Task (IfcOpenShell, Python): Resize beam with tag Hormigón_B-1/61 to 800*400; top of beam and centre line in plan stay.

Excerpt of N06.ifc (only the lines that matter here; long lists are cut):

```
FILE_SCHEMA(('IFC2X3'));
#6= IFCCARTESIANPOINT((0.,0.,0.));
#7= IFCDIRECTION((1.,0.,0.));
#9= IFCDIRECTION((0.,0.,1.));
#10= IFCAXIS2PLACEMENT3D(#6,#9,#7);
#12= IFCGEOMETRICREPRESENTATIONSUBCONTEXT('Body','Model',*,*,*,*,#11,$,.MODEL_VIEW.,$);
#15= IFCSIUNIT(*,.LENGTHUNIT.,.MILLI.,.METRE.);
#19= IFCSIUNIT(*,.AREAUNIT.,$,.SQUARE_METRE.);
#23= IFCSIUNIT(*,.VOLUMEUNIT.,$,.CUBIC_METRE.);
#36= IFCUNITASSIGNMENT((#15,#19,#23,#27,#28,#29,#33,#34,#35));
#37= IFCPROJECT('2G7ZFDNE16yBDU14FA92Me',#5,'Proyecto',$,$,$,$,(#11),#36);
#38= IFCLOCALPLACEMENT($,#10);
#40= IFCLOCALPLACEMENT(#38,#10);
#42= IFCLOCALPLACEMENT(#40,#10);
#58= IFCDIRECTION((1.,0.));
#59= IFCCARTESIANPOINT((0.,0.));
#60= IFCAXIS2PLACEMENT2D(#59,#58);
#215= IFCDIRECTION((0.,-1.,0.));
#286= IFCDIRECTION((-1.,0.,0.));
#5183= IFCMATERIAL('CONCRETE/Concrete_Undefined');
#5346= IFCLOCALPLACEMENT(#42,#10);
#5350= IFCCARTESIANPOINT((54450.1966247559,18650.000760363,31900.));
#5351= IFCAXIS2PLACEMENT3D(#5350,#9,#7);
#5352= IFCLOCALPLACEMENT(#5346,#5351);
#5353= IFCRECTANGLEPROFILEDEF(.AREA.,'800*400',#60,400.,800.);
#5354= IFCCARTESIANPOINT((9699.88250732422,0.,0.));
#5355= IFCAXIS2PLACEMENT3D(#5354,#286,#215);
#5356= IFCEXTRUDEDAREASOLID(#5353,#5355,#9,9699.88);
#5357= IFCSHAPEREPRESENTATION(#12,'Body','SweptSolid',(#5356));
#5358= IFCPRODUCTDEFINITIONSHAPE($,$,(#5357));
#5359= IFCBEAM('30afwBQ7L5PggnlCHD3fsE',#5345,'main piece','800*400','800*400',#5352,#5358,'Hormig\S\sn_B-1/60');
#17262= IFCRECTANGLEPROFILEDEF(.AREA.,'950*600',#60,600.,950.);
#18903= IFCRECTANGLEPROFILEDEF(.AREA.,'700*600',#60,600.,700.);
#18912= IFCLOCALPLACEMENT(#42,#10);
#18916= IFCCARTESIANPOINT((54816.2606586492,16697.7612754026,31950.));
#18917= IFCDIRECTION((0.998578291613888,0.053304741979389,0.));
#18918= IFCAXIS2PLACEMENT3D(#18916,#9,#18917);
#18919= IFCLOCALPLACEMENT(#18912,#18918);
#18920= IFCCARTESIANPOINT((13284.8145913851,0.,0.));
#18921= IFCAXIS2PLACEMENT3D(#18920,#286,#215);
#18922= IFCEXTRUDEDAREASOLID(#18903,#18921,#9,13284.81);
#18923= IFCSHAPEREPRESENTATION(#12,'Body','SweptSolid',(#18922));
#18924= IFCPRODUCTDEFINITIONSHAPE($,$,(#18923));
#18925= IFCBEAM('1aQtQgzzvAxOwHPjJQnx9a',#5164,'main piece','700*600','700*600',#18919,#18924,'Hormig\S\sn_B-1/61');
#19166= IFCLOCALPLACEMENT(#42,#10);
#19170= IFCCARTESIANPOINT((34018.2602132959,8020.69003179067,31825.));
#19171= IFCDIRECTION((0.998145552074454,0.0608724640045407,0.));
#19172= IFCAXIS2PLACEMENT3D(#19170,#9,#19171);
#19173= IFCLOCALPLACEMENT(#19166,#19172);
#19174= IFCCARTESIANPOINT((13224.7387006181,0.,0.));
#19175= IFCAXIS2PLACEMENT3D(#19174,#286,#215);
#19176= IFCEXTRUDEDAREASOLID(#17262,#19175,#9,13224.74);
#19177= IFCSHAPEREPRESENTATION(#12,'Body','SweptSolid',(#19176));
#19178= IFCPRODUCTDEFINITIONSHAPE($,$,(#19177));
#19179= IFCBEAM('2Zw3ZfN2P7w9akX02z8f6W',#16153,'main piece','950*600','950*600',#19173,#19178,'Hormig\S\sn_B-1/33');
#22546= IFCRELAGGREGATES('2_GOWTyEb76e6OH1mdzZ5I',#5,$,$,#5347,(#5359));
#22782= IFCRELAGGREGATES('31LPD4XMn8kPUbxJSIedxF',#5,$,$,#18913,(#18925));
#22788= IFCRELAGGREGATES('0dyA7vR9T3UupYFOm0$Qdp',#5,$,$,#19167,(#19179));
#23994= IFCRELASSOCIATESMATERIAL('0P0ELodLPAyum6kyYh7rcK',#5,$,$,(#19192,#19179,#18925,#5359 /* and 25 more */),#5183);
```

```python
import ifcopenshell
import ifcopenshell.util.element
import ifcopenshell.util.representation

model = ifcopenshell.open("N06.ifc")

member = model.by_guid("1aQtQgzzvAxOwHPjJQnx9a")
source = next(p for p in model.by_type("IfcRectangleProfileDef") if p.ProfileName == "800*400")

body = ifcopenshell.util.representation.get_representation(member, "Model", "Body")
solid = body.Items[0]
old_profile = solid.SweptArea

# Copy the section's sizes but keep this member's own profile position.
profile = ifcopenshell.util.element.copy(model, source)
# Profiles are centred, so shift by half the change in depth to hold the top.
shift = (old_profile.YDim - profile.YDim) / 2
x, y = old_profile.Position.Location.Coordinates
up = (0.0, 1.0)  # upwards, in the solid's own plane
location = model.createIfcCartesianPoint((x + up[0] * shift, y + up[1] * shift))
profile.Position = model.createIfcAxis2Placement2D(location, old_profile.Position.RefDirection)
solid.SweptArea = profile
if not model.get_total_inverses(old_profile):
    ifcopenshell.util.element.remove_deep2(model, old_profile)
member.Description = member.Description.replace("700*600", "800*400")
member.ObjectType = member.ObjectType.replace("700*600", "800*400")

print(solid.SweptArea)

model.write("N06_v2.ifc")
```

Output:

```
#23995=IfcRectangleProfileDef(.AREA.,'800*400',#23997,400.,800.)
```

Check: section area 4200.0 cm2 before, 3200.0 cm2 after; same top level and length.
